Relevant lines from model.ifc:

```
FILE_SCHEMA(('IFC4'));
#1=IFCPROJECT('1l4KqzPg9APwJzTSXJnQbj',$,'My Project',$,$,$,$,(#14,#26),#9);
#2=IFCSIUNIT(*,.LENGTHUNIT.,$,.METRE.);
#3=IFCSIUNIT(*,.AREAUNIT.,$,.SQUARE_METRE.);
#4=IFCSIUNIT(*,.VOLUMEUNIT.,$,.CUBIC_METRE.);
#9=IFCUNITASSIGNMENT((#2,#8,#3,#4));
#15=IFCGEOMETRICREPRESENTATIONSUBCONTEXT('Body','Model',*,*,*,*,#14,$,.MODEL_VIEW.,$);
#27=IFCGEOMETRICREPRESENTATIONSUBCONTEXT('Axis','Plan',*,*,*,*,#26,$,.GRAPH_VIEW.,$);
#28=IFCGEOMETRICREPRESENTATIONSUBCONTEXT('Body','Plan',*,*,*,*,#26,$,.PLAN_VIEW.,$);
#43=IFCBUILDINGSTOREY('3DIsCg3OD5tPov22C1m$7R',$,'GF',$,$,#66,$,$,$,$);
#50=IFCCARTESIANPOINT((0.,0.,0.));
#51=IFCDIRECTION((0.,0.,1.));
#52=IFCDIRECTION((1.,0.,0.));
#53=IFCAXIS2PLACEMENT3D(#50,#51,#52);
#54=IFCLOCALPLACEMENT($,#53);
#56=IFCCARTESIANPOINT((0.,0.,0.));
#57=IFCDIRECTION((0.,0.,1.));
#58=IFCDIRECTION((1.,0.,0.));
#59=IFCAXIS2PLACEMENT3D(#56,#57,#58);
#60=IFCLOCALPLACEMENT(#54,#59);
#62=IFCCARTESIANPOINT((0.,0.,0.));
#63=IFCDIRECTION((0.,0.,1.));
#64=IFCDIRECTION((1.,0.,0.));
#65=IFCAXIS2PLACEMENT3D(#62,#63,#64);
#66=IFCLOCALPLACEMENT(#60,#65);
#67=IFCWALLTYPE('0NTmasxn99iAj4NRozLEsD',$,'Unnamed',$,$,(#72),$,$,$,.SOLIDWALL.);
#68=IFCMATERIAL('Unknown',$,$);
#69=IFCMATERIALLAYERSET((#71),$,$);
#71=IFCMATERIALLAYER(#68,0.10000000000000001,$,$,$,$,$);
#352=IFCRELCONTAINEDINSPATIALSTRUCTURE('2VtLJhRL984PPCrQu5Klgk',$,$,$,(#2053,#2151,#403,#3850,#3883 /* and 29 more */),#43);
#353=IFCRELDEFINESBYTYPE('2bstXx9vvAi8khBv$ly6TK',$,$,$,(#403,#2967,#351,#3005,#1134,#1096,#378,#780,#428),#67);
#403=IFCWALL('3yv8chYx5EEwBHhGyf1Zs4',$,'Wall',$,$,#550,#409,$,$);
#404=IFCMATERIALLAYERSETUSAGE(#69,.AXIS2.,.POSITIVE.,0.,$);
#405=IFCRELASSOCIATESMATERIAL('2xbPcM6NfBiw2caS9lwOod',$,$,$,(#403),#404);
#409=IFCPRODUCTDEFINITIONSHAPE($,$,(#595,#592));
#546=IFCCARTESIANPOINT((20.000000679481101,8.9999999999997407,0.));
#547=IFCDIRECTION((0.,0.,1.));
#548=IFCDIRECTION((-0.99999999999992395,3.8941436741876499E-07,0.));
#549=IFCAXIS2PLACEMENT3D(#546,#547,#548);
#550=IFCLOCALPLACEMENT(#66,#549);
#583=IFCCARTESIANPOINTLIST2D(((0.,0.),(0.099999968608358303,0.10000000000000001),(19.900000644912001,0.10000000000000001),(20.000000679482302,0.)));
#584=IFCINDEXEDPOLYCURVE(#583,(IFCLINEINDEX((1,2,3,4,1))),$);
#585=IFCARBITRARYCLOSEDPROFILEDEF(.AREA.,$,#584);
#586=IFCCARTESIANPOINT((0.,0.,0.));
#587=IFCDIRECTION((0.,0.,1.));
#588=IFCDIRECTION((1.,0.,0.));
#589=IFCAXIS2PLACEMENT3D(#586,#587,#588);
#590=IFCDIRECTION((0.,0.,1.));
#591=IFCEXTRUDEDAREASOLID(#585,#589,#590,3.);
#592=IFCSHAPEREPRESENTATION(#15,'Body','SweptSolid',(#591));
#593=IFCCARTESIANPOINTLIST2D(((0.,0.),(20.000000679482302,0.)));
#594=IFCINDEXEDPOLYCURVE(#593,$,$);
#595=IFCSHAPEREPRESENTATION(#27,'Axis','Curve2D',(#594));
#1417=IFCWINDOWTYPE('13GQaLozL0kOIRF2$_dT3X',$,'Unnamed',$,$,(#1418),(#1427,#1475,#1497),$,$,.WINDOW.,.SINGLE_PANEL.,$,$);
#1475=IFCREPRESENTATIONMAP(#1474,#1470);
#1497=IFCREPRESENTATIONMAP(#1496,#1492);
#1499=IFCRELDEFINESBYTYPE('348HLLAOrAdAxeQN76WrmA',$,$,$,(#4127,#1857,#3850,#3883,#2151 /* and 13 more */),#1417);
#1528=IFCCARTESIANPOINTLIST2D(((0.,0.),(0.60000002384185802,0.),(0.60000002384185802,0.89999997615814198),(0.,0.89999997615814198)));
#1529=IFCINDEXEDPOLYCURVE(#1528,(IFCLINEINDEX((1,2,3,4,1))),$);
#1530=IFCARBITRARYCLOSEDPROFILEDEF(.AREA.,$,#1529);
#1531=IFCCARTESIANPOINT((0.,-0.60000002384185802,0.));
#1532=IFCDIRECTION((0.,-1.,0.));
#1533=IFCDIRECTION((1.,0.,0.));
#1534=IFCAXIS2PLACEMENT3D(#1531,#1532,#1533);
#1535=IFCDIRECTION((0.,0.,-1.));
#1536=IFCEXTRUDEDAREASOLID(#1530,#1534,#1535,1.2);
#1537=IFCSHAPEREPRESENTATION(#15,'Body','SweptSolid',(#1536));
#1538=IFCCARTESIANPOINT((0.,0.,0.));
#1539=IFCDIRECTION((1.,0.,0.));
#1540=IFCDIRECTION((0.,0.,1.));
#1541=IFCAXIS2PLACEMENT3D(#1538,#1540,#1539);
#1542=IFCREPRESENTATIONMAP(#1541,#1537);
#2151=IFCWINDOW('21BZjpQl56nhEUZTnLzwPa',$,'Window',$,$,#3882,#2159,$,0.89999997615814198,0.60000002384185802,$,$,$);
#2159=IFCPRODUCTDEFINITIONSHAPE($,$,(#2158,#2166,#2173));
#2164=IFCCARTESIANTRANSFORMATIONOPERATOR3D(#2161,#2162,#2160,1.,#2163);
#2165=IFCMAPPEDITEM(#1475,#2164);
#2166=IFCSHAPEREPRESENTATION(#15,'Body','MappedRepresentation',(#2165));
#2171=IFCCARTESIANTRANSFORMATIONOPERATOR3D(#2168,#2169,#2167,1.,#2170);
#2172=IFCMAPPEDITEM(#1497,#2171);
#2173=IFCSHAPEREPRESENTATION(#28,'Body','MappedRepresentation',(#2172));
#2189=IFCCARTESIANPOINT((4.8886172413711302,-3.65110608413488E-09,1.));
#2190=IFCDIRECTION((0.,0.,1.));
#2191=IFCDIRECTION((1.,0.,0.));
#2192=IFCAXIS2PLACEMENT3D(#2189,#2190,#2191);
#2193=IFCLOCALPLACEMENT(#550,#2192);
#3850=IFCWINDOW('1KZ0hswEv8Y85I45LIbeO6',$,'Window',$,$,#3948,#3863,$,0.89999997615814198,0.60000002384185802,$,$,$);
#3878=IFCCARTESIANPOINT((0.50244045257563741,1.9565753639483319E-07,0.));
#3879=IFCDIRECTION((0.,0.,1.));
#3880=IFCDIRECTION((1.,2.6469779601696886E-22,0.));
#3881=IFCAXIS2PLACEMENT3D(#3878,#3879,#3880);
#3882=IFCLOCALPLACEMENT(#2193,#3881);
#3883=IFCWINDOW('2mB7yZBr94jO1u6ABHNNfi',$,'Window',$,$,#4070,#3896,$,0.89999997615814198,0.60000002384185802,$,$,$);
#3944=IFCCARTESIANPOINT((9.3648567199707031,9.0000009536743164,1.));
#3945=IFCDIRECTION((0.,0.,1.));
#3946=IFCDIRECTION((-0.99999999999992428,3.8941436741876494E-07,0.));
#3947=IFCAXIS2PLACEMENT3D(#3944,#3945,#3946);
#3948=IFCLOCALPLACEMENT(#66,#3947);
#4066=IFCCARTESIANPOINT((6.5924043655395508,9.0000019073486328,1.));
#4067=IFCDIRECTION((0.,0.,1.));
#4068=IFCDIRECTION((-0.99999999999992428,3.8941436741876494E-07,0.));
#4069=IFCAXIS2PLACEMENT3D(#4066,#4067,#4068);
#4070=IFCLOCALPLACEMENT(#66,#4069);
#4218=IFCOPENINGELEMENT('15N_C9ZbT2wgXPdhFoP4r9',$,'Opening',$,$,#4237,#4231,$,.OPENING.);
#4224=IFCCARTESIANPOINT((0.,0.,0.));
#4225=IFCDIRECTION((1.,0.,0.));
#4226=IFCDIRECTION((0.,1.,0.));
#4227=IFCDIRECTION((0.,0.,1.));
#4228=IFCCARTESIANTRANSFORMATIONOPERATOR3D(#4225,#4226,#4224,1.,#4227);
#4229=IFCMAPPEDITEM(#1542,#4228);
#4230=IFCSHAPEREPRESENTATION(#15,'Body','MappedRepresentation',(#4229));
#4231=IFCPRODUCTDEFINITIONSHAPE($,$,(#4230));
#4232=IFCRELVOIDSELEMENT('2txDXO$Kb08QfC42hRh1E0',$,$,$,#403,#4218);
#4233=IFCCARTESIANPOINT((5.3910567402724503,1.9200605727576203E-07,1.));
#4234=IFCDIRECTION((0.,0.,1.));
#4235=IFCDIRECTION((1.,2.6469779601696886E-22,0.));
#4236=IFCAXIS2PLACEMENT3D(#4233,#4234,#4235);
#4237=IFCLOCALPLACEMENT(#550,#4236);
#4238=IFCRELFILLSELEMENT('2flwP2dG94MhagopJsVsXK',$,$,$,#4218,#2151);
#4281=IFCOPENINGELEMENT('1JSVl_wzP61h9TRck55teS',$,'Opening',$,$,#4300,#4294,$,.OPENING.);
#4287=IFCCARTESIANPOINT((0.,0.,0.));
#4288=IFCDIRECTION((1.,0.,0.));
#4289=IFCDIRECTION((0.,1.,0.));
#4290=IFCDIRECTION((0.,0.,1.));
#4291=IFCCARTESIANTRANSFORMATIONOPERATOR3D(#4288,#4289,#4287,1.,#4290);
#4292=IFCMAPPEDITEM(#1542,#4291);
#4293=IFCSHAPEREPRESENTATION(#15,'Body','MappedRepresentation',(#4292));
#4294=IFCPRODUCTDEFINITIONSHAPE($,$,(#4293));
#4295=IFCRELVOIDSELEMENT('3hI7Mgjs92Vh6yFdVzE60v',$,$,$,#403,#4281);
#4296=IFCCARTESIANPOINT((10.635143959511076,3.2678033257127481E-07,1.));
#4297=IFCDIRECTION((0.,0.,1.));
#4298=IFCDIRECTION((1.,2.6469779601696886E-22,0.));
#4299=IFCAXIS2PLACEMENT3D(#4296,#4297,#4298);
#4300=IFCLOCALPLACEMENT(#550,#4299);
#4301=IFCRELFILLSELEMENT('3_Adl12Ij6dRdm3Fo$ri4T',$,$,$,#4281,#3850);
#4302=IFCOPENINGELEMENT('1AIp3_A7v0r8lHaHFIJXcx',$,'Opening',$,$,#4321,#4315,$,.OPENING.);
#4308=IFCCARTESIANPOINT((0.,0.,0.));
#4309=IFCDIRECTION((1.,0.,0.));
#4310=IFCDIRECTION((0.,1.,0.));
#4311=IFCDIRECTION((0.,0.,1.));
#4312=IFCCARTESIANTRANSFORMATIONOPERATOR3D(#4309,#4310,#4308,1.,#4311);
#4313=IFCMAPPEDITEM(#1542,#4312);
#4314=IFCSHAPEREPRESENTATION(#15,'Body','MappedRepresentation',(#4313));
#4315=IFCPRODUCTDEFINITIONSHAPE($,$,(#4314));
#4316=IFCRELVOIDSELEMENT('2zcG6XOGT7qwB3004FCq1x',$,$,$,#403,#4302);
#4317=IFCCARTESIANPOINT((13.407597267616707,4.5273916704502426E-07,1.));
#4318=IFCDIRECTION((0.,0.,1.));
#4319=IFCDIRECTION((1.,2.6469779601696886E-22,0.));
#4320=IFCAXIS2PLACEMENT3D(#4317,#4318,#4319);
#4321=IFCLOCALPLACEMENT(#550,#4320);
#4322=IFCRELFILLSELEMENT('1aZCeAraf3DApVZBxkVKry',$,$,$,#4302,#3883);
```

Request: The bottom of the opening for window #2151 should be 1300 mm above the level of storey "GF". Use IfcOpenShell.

```python
import numpy as np
import ifcopenshell
import ifcopenshell.api.geometry
import ifcopenshell.geom
import ifcopenshell.util.element
import ifcopenshell.util.placement
import ifcopenshell.util.shape
import ifcopenshell.util.unit

model = ifcopenshell.open("model.ifc")
unit_scale = ifcopenshell.util.unit.calculate_unit_scale(model)

window = model.by_id(2151)
opening = window.FillsVoids[0].RelatingOpeningElement
storey = ifcopenshell.util.element.get_container(window, ifc_class="IfcBuildingStorey")
level = ifcopenshell.util.placement.get_local_placement(storey.ObjectPlacement)[2, 3]

# The opening's origin need not be at the sill, so measure its lowest point.
shape = ifcopenshell.geom.create_shape(ifcopenshell.geom.settings(), opening)
bottom = ifcopenshell.util.shape.get_shape_bottom_elevation(shape, shape.geometry) / unit_scale
dz = level + 1.3 / unit_scale - bottom

shift = np.array([0.0, 0.0, dz])
# The window is not placed relative to its opening, so move both.
for product in (opening, window):
    matrix = ifcopenshell.util.placement.get_local_placement(product.ObjectPlacement)
    matrix[:3, 3] += shift
    ifcopenshell.api.geometry.edit_object_placement(model, product=product, matrix=matrix, is_si=False)

print(f"moved by {dz * unit_scale:+.3f} m")

model.write("model_updated.ifc")
```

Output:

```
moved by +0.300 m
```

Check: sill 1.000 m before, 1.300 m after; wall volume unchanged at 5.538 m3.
